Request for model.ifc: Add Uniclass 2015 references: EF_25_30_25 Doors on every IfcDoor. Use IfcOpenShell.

First a look at what the model holds.

```python
import ifcopenshell

model = ifcopenshell.open("model.ifc")
print(model.schema)
print("classifications:", [c.Name for c in model.by_type("IfcClassification")])
for ifc_class in ("IfcDoor", "IfcRoof", "IfcStair", "IfcWall", "IfcWindow"):
    print(ifc_class, len(model.by_type(ifc_class)))
```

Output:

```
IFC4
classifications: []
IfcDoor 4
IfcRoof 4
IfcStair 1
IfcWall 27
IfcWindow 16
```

```python
import ifcopenshell
import ifcopenshell.api.classification

model = ifcopenshell.open("model.ifc")

system = ifcopenshell.api.classification.add_classification(model, classification="Uniclass 2015")

codes = {
    "IfcDoor": ("EF_25_30_25", "Doors"),
}
for ifc_class, (code, name) in codes.items():
    products = model.by_type(ifc_class)
    ifcopenshell.api.classification.add_reference(
        model, products=products, classification=system, identification=code, name=name
    )
    print(code, len(products))

model.write("model_v2.ifc")
```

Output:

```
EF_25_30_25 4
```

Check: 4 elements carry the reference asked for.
